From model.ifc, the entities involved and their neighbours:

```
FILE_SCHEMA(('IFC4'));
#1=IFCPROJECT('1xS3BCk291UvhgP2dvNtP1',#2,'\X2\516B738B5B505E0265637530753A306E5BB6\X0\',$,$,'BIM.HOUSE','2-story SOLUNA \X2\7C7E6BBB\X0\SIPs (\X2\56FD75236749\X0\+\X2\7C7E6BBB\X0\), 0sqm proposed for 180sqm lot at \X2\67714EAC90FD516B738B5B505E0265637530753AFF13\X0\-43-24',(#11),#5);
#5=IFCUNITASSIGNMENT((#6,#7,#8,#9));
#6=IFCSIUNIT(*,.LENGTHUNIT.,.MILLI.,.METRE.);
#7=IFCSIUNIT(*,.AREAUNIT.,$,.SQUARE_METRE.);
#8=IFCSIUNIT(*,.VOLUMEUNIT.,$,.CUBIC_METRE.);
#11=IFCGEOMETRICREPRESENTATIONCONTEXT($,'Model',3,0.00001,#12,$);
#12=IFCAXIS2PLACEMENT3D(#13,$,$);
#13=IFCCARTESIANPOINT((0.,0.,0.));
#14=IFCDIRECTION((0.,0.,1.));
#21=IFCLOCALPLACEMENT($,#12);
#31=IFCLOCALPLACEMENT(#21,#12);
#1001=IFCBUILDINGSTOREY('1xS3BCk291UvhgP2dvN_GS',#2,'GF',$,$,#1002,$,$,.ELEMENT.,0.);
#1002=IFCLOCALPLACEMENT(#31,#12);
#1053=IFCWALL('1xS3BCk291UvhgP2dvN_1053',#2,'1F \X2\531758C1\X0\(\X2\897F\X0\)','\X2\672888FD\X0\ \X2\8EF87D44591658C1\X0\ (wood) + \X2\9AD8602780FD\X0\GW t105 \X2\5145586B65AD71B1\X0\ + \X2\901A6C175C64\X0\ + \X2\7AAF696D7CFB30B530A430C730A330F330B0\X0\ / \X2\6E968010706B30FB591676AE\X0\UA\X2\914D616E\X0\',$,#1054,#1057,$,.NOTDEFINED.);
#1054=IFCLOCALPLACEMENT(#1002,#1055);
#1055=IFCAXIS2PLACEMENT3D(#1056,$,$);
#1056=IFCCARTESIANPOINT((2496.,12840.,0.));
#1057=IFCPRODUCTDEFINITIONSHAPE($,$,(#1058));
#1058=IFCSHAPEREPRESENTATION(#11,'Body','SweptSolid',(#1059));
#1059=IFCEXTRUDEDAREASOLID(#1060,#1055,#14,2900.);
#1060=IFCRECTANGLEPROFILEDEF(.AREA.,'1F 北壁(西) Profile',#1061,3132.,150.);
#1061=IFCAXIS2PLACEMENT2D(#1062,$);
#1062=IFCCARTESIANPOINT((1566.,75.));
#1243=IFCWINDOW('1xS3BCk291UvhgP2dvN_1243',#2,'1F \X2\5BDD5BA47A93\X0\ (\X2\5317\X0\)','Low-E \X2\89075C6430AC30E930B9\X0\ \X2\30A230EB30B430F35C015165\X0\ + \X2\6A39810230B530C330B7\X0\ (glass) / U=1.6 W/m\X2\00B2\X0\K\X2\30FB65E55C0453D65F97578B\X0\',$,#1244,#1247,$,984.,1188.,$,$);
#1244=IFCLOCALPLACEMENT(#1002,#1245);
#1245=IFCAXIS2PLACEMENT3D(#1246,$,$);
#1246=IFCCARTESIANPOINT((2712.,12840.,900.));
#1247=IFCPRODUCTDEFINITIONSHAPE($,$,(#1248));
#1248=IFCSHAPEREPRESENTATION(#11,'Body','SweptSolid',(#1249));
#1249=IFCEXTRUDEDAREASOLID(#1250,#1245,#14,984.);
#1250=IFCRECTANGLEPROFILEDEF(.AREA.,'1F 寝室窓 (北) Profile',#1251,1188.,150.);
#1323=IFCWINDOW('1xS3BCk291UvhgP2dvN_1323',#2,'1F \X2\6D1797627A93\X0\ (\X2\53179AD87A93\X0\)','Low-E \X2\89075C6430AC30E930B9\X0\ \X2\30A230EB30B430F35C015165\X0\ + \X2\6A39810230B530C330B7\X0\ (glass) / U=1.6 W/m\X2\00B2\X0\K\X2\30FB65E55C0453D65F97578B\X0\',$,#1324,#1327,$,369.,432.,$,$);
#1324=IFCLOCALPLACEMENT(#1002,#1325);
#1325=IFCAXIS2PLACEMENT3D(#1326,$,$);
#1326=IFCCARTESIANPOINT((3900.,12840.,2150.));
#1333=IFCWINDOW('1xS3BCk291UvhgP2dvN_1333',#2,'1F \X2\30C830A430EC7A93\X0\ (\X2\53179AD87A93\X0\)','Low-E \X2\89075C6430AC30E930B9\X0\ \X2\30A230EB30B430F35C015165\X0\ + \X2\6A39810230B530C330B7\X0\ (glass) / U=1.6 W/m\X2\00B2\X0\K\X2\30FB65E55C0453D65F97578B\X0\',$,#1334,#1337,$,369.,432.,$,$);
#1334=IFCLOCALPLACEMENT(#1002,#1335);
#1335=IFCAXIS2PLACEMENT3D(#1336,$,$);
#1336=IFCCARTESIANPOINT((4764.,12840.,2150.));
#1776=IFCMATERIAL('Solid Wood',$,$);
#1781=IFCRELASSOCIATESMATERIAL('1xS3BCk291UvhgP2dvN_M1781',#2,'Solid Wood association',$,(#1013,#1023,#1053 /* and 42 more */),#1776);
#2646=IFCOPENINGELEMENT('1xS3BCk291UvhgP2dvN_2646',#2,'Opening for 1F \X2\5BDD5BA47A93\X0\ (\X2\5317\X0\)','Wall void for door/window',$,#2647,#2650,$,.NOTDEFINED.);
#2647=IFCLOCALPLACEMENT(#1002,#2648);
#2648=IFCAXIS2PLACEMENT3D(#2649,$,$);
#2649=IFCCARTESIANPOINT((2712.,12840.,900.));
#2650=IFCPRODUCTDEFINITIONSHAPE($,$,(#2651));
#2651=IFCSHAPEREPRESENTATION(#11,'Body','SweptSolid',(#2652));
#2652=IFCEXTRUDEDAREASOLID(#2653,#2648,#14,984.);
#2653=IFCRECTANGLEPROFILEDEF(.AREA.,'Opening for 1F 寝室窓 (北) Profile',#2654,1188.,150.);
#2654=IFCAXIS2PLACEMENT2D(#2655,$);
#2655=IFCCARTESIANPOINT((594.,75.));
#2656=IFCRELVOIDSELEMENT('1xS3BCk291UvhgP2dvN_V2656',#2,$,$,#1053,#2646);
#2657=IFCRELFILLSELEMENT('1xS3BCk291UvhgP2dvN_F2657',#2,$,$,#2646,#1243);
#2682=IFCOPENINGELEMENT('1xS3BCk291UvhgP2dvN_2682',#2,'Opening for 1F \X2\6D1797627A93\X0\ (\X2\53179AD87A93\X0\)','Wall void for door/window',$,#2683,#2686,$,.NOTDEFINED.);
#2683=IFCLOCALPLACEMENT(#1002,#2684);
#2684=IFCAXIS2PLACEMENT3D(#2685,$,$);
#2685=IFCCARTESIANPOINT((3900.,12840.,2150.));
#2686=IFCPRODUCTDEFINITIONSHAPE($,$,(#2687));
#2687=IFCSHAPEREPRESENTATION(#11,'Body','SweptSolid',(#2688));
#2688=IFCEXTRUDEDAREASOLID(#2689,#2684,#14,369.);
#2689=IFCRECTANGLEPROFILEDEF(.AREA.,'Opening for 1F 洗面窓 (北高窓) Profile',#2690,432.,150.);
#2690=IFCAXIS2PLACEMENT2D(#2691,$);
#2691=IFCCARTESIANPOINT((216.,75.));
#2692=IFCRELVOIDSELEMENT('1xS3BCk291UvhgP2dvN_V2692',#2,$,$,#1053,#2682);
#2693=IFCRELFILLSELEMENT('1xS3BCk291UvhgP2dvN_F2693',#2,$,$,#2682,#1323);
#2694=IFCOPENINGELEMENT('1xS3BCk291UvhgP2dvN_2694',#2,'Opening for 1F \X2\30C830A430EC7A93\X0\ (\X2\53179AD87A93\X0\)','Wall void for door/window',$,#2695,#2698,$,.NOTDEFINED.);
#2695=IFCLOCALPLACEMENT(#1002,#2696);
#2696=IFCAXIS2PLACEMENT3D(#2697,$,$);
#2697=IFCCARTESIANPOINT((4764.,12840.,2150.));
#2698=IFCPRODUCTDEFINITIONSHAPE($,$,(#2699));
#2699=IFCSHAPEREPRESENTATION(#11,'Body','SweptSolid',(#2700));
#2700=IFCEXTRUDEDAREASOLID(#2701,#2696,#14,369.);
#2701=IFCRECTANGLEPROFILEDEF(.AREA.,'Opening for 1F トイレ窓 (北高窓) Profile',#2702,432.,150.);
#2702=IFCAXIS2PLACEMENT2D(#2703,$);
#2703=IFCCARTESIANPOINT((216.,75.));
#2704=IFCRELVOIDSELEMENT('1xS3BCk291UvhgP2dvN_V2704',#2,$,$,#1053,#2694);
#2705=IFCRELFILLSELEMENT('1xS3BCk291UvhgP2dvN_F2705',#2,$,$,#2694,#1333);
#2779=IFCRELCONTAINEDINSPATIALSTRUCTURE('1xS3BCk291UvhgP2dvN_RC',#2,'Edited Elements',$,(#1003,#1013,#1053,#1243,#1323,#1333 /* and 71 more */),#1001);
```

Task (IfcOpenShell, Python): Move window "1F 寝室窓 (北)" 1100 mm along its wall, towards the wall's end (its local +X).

```python
import ifcopenshell
import ifcopenshell.api.geometry
import ifcopenshell.util.placement
import ifcopenshell.util.unit

model = ifcopenshell.open("model.ifc")
unit_scale = ifcopenshell.util.unit.calculate_unit_scale(model)

window = model.by_id(1243)
opening = window.FillsVoids[0].RelatingOpeningElement
wall = opening.VoidsElements[0].RelatingBuildingElement

wall_matrix = ifcopenshell.util.placement.get_local_placement(wall.ObjectPlacement)
shift = wall_matrix[:3, 0] * 1.1 / unit_scale
before = ifcopenshell.util.placement.get_local_placement(window.ObjectPlacement)[:3, 3].copy()

# The window is not placed relative to its opening, so move both.
for product in (opening, window):
    matrix = ifcopenshell.util.placement.get_local_placement(product.ObjectPlacement)
    matrix[:3, 3] += shift
    ifcopenshell.api.geometry.edit_object_placement(model, product=product, matrix=matrix, is_si=False)

after = ifcopenshell.util.placement.get_local_placement(window.ObjectPlacement)[:3, 3]
print("window moved by", (after - before).round(3) + 0.0)

model.write("model_updated.ifc")
```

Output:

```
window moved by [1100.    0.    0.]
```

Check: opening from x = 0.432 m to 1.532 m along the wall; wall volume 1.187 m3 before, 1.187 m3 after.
